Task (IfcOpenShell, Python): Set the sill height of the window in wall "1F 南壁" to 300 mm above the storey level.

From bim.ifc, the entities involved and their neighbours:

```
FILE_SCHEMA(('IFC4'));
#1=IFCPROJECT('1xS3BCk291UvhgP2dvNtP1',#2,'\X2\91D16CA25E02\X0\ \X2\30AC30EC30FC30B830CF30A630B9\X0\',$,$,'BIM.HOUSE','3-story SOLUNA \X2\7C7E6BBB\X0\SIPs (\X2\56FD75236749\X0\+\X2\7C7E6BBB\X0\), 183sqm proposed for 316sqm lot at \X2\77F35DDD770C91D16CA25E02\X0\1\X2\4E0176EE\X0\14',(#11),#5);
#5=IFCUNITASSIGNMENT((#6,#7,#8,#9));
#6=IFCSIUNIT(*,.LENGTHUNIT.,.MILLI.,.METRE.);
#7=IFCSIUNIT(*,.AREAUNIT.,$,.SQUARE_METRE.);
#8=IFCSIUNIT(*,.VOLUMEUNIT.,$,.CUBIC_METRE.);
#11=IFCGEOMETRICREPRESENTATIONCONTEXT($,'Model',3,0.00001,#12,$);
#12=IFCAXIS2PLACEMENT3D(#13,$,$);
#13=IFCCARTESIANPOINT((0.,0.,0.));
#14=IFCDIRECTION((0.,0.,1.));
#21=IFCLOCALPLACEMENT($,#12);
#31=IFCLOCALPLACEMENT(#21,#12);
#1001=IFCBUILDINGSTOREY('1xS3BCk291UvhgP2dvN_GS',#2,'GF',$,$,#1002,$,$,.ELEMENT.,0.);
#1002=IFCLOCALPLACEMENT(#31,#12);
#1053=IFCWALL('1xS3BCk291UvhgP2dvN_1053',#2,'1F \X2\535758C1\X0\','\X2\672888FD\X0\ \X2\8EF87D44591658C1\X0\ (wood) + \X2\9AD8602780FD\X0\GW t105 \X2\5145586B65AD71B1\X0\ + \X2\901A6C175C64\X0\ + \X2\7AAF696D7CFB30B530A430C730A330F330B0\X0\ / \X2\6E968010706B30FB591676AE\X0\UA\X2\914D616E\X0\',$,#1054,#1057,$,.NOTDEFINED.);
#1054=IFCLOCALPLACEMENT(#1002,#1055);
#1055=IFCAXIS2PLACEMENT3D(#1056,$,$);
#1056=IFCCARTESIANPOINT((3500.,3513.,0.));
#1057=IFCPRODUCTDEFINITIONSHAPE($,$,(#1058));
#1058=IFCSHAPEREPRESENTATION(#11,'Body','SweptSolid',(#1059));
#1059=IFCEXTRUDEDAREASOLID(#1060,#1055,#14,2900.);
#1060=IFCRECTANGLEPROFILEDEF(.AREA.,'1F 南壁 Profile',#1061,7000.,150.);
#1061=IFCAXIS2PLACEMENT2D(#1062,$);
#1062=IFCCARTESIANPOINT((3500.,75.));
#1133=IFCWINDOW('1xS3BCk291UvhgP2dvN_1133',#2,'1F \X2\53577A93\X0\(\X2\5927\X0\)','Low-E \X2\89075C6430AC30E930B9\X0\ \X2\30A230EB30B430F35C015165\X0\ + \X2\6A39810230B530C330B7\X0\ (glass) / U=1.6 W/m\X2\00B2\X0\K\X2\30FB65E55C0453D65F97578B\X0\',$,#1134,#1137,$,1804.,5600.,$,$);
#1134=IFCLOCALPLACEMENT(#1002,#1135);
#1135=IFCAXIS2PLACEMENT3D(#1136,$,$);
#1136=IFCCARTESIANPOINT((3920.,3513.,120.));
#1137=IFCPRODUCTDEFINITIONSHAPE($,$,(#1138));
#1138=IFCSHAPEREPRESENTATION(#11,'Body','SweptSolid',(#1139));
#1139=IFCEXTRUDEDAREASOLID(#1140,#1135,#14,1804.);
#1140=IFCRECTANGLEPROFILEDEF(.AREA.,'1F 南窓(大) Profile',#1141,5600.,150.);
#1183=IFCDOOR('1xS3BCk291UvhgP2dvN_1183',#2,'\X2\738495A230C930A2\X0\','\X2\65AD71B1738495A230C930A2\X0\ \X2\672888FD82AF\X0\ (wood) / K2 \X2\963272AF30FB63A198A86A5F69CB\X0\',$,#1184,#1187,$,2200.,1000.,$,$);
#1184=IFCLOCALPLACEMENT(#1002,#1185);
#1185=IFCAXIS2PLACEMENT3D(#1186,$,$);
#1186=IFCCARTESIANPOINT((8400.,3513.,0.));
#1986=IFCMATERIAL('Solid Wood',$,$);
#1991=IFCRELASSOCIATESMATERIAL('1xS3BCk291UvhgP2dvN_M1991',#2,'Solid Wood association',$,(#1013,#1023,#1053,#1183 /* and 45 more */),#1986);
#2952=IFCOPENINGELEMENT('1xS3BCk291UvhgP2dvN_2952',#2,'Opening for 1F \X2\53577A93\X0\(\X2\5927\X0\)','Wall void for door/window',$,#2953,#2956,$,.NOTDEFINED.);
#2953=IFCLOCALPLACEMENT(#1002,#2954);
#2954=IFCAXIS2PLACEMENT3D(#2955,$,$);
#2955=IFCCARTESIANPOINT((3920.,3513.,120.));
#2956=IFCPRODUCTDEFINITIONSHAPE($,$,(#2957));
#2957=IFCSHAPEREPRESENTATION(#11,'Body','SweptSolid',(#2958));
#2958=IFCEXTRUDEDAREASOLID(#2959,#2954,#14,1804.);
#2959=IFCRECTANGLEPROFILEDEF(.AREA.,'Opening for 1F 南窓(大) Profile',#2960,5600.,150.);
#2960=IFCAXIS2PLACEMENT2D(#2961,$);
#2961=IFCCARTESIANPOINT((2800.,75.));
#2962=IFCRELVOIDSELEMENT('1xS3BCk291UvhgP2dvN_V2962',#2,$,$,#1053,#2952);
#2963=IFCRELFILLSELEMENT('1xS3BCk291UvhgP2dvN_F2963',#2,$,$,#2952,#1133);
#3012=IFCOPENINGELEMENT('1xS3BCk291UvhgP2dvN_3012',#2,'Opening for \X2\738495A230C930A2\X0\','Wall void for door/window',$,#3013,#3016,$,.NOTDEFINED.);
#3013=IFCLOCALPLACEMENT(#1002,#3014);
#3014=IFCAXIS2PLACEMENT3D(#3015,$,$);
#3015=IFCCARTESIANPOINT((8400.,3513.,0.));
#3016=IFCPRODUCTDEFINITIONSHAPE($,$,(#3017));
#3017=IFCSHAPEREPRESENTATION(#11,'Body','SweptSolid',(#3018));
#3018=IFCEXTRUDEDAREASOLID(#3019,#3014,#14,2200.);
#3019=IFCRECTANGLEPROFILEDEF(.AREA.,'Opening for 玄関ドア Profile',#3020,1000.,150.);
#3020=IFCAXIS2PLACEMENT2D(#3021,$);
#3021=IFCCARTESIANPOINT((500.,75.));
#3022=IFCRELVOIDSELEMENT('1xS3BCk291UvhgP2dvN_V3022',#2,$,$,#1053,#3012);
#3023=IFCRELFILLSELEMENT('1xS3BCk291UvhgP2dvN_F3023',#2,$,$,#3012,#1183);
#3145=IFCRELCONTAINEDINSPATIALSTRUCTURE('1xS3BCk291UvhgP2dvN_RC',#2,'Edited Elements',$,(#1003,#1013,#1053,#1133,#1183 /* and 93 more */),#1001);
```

```python
import numpy as np
import ifcopenshell
import ifcopenshell.api.geometry
import ifcopenshell.geom
import ifcopenshell.util.element
import ifcopenshell.util.placement
import ifcopenshell.util.shape
import ifcopenshell.util.unit

model = ifcopenshell.open("bim.ifc")
unit_scale = ifcopenshell.util.unit.calculate_unit_scale(model)

window = model.by_id(1133)
opening = window.FillsVoids[0].RelatingOpeningElement
storey = ifcopenshell.util.element.get_container(window, ifc_class="IfcBuildingStorey")
level = ifcopenshell.util.placement.get_local_placement(storey.ObjectPlacement)[2, 3]

# The opening's origin need not be at the sill, so measure its lowest point.
shape = ifcopenshell.geom.create_shape(ifcopenshell.geom.settings(), opening)
bottom = ifcopenshell.util.shape.get_shape_bottom_elevation(shape, shape.geometry) / unit_scale
dz = level + 300.0 - bottom

shift = np.array([0.0, 0.0, dz])
# The window is not placed relative to its opening, so move both.
for product in (opening, window):
    matrix = ifcopenshell.util.placement.get_local_placement(product.ObjectPlacement)
    matrix[:3, 3] += shift
    ifcopenshell.api.geometry.edit_object_placement(model, product=product, matrix=matrix, is_si=False)

print(f"moved by {dz * unit_scale:+.3f} m")

model.write("bim-out.ifc")
```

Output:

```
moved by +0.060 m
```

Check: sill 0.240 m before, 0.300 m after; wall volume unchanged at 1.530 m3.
